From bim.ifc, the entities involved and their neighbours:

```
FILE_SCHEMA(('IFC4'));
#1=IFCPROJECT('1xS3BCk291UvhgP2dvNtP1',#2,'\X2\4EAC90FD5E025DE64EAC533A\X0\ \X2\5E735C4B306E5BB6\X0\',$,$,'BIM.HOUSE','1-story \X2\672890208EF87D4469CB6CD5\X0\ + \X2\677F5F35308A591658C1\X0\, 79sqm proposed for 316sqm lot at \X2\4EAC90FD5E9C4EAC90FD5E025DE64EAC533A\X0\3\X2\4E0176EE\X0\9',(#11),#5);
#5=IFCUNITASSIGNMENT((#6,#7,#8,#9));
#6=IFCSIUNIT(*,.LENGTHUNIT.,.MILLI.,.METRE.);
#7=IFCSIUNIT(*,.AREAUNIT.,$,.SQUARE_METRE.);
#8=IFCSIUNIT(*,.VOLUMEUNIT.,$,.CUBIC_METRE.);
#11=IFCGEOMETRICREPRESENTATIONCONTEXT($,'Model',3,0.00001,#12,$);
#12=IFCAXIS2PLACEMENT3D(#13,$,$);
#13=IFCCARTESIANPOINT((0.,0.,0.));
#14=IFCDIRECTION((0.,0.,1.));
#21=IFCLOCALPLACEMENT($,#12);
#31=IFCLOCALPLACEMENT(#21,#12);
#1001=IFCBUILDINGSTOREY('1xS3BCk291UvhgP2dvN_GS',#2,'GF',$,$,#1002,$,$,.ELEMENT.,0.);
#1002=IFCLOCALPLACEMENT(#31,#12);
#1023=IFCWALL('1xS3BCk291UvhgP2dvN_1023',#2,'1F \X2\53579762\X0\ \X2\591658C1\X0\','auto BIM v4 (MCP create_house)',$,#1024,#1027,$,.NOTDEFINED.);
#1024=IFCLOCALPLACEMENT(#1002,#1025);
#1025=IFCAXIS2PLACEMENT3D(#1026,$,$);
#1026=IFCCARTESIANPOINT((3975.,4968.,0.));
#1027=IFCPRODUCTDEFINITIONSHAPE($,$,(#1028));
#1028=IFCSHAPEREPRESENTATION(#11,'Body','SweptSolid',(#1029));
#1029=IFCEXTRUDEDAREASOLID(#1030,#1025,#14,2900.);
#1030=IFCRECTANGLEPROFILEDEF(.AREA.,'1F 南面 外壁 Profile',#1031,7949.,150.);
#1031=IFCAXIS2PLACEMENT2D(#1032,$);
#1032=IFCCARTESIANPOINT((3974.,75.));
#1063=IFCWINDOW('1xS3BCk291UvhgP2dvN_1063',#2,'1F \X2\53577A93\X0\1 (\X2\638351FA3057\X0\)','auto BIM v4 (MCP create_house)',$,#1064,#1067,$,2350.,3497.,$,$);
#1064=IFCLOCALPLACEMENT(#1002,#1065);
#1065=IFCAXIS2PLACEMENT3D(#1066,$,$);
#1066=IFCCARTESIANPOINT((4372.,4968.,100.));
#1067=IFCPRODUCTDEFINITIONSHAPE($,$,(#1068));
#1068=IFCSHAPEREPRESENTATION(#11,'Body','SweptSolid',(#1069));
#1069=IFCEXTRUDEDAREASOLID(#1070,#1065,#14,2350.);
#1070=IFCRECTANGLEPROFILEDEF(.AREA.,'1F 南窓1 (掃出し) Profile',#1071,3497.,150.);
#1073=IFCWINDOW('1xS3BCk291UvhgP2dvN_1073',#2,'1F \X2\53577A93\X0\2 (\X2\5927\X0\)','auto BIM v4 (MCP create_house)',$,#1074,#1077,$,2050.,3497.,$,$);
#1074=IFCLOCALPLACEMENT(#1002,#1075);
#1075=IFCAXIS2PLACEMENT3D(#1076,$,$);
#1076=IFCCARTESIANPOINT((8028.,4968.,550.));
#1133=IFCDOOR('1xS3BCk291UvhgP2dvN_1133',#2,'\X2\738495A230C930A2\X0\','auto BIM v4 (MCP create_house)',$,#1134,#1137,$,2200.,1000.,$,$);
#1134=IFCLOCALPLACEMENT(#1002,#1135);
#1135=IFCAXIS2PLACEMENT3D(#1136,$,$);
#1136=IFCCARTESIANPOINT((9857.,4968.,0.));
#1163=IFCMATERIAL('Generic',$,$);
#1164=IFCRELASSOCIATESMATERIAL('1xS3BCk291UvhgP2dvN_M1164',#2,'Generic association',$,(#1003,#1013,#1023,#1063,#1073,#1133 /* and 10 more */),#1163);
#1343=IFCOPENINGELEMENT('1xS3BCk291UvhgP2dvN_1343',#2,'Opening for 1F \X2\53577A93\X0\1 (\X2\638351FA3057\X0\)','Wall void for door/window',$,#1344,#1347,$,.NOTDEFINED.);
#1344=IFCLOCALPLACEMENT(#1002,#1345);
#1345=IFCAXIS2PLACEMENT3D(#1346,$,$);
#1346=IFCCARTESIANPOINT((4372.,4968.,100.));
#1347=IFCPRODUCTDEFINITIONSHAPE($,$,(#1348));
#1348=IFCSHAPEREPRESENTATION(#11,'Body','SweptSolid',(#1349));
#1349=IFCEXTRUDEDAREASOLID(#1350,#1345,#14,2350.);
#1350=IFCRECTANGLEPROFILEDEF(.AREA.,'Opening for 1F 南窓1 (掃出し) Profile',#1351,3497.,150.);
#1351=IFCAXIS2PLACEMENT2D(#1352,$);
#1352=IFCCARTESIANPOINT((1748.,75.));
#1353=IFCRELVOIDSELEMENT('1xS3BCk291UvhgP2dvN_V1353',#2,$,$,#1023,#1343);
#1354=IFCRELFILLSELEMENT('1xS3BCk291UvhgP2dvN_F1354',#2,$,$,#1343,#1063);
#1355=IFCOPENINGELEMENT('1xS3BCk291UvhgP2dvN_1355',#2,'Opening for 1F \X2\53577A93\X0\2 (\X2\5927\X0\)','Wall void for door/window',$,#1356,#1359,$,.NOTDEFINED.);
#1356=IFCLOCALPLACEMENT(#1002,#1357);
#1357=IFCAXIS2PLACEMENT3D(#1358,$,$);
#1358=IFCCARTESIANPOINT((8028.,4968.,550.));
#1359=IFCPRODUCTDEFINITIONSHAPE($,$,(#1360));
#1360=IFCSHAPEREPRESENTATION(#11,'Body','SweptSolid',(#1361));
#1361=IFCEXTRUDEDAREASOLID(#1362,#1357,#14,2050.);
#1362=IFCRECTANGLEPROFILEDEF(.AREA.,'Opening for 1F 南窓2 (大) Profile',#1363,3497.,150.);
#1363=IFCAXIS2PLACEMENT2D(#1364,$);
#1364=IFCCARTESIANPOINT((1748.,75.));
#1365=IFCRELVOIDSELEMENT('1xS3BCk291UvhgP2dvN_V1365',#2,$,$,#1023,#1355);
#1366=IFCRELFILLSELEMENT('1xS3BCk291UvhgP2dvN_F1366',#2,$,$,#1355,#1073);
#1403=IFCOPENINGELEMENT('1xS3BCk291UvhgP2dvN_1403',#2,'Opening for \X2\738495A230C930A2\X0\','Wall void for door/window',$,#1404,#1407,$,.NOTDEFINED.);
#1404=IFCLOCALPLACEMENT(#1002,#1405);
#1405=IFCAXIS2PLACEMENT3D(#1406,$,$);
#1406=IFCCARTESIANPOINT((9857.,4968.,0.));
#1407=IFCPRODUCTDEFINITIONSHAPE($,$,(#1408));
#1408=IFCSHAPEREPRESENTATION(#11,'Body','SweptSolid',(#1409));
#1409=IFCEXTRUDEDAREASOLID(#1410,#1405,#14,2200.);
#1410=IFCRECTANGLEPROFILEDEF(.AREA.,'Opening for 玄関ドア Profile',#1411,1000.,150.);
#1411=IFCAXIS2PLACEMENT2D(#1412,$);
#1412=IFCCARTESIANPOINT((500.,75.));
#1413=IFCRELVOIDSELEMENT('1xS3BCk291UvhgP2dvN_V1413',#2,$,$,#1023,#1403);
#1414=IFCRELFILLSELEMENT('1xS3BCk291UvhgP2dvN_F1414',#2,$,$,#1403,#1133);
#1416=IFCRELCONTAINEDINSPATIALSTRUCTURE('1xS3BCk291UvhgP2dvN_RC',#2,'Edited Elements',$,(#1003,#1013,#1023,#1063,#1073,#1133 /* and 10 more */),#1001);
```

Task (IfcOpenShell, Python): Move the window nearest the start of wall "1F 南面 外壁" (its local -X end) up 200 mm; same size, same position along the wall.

```python
import numpy as np
import ifcopenshell
import ifcopenshell.api.geometry
import ifcopenshell.util.placement
import ifcopenshell.util.unit

model = ifcopenshell.open("bim.ifc")
unit_scale = ifcopenshell.util.unit.calculate_unit_scale(model)

window = model.by_guid("1xS3BCk291UvhgP2dvN_1063")
opening = window.FillsVoids[0].RelatingOpeningElement
dz = 0.2 / unit_scale

shift = np.array([0.0, 0.0, dz])
# The window is not placed relative to its opening, so move both.
for product in (opening, window):
    matrix = ifcopenshell.util.placement.get_local_placement(product.ObjectPlacement)
    matrix[:3, 3] += shift
    ifcopenshell.api.geometry.edit_object_placement(model, product=product, matrix=matrix, is_si=False)

print(f"moved by {dz * unit_scale:+.3f} m")

model.write("bim_rev.ifc")
```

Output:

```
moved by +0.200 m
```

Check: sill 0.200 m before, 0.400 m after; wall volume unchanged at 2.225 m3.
